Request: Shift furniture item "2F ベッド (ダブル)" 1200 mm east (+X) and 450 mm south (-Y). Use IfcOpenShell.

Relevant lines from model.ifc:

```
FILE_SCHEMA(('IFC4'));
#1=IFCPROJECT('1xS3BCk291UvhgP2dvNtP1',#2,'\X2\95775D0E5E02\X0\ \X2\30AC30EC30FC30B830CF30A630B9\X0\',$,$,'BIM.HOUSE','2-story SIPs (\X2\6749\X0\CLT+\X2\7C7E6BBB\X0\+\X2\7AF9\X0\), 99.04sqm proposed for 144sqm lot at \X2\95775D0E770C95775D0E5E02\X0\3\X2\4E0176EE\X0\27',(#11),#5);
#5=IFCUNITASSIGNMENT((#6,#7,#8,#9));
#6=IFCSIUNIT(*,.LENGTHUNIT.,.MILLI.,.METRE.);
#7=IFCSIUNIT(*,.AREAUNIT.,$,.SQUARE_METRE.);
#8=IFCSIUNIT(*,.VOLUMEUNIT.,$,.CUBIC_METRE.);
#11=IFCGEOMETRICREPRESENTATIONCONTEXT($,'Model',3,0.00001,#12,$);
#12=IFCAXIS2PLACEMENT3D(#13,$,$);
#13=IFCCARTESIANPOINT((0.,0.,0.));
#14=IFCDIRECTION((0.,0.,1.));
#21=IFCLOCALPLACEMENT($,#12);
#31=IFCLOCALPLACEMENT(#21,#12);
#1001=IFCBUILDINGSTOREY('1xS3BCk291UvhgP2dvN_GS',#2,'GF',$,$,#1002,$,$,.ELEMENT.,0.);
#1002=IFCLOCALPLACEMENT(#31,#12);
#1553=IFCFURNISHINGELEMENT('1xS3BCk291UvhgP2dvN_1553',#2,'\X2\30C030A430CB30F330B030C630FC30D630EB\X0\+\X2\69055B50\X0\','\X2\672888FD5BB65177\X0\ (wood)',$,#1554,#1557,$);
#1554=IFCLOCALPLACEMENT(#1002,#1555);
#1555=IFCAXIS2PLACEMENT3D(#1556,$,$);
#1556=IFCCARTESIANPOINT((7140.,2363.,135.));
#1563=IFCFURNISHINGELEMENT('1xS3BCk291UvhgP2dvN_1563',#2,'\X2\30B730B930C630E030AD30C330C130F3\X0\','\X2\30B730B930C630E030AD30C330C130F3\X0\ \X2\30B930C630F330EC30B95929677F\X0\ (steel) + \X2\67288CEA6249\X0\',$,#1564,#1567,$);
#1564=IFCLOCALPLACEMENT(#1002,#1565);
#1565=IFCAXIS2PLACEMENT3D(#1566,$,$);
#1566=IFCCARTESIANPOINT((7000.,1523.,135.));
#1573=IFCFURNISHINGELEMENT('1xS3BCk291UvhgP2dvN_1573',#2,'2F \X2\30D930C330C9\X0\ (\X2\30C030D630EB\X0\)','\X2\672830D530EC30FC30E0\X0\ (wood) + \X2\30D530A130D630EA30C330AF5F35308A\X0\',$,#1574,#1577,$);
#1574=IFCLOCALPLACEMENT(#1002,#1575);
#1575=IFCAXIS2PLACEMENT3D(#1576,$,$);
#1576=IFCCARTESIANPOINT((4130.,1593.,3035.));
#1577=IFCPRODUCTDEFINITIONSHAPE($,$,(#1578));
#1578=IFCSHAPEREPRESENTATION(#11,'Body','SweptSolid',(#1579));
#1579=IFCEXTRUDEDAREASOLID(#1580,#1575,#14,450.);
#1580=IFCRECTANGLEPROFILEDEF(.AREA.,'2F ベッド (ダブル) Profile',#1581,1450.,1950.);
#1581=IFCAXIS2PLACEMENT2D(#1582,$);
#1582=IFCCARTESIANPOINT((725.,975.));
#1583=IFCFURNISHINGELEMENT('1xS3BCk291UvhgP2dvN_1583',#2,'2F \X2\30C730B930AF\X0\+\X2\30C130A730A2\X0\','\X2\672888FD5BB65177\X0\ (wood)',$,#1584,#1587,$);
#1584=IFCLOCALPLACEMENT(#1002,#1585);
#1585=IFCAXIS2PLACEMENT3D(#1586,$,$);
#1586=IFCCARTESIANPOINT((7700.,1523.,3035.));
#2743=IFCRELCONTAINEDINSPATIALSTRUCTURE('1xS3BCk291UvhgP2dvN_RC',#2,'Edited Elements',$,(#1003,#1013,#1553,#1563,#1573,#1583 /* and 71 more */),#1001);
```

```python
import ifcopenshell
import ifcopenshell.api.geometry
import ifcopenshell.util.placement
import ifcopenshell.util.unit

model = ifcopenshell.open("model.ifc")
unit_scale = ifcopenshell.util.unit.calculate_unit_scale(model)

item = model.by_guid("1xS3BCk291UvhgP2dvN_1573")
matrix = ifcopenshell.util.placement.get_local_placement(item.ObjectPlacement)
matrix[0, 3] += 1.2 / unit_scale
matrix[1, 3] -= 0.45 / unit_scale
ifcopenshell.api.geometry.edit_object_placement(model, product=item, matrix=matrix, is_si=False)

print(ifcopenshell.util.placement.get_local_placement(item.ObjectPlacement).round(3) + 0.0)

model.write("model_rev.ifc")
```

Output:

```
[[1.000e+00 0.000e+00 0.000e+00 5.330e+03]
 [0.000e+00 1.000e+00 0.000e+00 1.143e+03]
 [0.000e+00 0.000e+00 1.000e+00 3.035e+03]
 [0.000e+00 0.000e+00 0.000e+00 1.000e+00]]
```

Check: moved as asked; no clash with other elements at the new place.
